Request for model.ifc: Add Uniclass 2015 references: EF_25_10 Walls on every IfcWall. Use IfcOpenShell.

First a look at what the model holds.

```python
import ifcopenshell

model = ifcopenshell.open("model.ifc")
print(model.schema)
print("classifications:", [c.Name for c in model.by_type("IfcClassification")])
for ifc_class in ("IfcDoor", "IfcRoof", "IfcStair", "IfcWall", "IfcWindow"):
    print(ifc_class, len(model.by_type(ifc_class)))
```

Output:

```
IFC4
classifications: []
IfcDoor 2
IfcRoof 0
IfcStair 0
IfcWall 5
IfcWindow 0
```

```python
import ifcopenshell
import ifcopenshell.api.classification

model = ifcopenshell.open("model.ifc")

system = ifcopenshell.api.classification.add_classification(model, classification="Uniclass 2015")

codes = {
    "IfcWall": ("EF_25_10", "Walls"),
}
for ifc_class, (code, name) in codes.items():
    products = model.by_type(ifc_class)
    ifcopenshell.api.classification.add_reference(
        model, products=products, classification=system, identification=code, name=name
    )
    print(code, len(products))

model.write("model_rev.ifc")
```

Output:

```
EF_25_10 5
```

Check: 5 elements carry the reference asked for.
